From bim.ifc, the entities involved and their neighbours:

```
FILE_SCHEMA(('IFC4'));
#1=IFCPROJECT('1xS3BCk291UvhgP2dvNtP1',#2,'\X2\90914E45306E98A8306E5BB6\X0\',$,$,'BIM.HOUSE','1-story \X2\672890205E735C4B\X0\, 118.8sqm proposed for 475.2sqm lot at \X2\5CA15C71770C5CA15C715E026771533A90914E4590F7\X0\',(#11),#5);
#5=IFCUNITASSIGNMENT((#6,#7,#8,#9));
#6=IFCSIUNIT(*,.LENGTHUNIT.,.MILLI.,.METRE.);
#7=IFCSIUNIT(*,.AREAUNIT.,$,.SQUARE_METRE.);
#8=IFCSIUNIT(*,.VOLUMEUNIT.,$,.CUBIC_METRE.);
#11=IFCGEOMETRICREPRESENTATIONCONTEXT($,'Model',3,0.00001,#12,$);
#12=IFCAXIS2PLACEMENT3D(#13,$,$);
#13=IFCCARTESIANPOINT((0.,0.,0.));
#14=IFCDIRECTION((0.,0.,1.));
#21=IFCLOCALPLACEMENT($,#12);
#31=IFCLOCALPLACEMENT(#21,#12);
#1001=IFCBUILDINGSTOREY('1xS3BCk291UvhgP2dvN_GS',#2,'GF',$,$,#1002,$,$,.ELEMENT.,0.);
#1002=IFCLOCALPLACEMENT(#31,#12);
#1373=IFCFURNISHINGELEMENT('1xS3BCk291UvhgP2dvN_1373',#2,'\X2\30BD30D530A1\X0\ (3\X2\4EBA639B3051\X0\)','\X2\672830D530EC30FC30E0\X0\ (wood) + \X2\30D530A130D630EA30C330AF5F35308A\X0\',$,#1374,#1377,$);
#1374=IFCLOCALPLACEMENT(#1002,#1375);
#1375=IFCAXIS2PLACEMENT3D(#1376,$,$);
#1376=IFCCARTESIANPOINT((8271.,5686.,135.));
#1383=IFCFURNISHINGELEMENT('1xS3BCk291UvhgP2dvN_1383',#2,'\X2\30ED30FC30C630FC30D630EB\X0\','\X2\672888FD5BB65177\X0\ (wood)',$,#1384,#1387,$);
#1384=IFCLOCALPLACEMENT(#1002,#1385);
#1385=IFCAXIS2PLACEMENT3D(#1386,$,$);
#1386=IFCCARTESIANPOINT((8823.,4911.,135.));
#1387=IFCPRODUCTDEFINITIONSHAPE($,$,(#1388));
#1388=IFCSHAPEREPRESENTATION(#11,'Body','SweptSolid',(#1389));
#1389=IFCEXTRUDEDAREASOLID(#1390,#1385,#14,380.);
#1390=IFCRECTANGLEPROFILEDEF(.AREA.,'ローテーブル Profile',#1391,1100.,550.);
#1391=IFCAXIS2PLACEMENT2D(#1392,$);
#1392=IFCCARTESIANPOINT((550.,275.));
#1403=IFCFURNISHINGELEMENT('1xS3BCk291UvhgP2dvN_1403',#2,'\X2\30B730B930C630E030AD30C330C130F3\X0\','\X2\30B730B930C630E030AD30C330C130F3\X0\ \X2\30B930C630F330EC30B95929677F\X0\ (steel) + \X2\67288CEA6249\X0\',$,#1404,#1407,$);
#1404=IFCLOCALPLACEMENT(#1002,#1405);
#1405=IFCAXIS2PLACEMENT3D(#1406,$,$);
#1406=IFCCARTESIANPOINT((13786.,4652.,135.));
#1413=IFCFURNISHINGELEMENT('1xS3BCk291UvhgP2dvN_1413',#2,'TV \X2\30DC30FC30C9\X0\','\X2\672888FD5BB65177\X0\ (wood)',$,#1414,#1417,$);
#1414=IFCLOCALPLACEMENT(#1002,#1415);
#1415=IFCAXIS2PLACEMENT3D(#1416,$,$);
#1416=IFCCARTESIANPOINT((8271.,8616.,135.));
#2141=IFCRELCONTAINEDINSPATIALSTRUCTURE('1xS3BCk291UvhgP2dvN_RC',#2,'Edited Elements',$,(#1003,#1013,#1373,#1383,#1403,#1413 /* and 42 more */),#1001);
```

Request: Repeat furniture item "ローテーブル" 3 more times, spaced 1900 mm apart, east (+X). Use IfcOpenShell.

```python
import numpy as np
import ifcopenshell
import ifcopenshell.api.geometry
import ifcopenshell.api.root
import ifcopenshell.util.element
import ifcopenshell.util.placement
import ifcopenshell.util.unit

model = ifcopenshell.open("bim.ifc")
unit_scale = ifcopenshell.util.unit.calculate_unit_scale(model)


def reuse_history(source, copy):
    """copy_class also copies each property set's owner history, people and application; keep the originals."""
    for rel in copy.IsDefinedBy:
        if rel.is_a("IfcRelDefinesByProperties") and (history := rel.RelatingPropertyDefinition.OwnerHistory):
            rel.RelatingPropertyDefinition.OwnerHistory = source.OwnerHistory
            ifcopenshell.util.element.remove_deep2(model, history)


source = model.by_guid("1xS3BCk291UvhgP2dvN_1383")
base = ifcopenshell.util.placement.get_local_placement(source.ObjectPlacement)
step = np.array([1.0, 0.0, 0.0]) * 1.9 / unit_scale

for i in range(1, 4):
    copy = ifcopenshell.api.root.copy_class(model, product=source)
    copy.Representation = ifcopenshell.util.element.copy_deep(
        model, source.Representation, exclude=["IfcGeometricRepresentationContext", "IfcRepresentationMap"]
    )
    reuse_history(source, copy)
    matrix = base.copy()
    matrix[:3, 3] += i * step
    print("added at", matrix[:3, 3].round(3) + 0.0)
    ifcopenshell.api.geometry.edit_object_placement(model, product=copy, matrix=matrix, is_si=False)

model.write("bim_v2.ifc")
```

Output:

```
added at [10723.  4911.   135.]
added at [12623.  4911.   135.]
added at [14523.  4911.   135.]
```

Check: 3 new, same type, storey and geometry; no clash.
